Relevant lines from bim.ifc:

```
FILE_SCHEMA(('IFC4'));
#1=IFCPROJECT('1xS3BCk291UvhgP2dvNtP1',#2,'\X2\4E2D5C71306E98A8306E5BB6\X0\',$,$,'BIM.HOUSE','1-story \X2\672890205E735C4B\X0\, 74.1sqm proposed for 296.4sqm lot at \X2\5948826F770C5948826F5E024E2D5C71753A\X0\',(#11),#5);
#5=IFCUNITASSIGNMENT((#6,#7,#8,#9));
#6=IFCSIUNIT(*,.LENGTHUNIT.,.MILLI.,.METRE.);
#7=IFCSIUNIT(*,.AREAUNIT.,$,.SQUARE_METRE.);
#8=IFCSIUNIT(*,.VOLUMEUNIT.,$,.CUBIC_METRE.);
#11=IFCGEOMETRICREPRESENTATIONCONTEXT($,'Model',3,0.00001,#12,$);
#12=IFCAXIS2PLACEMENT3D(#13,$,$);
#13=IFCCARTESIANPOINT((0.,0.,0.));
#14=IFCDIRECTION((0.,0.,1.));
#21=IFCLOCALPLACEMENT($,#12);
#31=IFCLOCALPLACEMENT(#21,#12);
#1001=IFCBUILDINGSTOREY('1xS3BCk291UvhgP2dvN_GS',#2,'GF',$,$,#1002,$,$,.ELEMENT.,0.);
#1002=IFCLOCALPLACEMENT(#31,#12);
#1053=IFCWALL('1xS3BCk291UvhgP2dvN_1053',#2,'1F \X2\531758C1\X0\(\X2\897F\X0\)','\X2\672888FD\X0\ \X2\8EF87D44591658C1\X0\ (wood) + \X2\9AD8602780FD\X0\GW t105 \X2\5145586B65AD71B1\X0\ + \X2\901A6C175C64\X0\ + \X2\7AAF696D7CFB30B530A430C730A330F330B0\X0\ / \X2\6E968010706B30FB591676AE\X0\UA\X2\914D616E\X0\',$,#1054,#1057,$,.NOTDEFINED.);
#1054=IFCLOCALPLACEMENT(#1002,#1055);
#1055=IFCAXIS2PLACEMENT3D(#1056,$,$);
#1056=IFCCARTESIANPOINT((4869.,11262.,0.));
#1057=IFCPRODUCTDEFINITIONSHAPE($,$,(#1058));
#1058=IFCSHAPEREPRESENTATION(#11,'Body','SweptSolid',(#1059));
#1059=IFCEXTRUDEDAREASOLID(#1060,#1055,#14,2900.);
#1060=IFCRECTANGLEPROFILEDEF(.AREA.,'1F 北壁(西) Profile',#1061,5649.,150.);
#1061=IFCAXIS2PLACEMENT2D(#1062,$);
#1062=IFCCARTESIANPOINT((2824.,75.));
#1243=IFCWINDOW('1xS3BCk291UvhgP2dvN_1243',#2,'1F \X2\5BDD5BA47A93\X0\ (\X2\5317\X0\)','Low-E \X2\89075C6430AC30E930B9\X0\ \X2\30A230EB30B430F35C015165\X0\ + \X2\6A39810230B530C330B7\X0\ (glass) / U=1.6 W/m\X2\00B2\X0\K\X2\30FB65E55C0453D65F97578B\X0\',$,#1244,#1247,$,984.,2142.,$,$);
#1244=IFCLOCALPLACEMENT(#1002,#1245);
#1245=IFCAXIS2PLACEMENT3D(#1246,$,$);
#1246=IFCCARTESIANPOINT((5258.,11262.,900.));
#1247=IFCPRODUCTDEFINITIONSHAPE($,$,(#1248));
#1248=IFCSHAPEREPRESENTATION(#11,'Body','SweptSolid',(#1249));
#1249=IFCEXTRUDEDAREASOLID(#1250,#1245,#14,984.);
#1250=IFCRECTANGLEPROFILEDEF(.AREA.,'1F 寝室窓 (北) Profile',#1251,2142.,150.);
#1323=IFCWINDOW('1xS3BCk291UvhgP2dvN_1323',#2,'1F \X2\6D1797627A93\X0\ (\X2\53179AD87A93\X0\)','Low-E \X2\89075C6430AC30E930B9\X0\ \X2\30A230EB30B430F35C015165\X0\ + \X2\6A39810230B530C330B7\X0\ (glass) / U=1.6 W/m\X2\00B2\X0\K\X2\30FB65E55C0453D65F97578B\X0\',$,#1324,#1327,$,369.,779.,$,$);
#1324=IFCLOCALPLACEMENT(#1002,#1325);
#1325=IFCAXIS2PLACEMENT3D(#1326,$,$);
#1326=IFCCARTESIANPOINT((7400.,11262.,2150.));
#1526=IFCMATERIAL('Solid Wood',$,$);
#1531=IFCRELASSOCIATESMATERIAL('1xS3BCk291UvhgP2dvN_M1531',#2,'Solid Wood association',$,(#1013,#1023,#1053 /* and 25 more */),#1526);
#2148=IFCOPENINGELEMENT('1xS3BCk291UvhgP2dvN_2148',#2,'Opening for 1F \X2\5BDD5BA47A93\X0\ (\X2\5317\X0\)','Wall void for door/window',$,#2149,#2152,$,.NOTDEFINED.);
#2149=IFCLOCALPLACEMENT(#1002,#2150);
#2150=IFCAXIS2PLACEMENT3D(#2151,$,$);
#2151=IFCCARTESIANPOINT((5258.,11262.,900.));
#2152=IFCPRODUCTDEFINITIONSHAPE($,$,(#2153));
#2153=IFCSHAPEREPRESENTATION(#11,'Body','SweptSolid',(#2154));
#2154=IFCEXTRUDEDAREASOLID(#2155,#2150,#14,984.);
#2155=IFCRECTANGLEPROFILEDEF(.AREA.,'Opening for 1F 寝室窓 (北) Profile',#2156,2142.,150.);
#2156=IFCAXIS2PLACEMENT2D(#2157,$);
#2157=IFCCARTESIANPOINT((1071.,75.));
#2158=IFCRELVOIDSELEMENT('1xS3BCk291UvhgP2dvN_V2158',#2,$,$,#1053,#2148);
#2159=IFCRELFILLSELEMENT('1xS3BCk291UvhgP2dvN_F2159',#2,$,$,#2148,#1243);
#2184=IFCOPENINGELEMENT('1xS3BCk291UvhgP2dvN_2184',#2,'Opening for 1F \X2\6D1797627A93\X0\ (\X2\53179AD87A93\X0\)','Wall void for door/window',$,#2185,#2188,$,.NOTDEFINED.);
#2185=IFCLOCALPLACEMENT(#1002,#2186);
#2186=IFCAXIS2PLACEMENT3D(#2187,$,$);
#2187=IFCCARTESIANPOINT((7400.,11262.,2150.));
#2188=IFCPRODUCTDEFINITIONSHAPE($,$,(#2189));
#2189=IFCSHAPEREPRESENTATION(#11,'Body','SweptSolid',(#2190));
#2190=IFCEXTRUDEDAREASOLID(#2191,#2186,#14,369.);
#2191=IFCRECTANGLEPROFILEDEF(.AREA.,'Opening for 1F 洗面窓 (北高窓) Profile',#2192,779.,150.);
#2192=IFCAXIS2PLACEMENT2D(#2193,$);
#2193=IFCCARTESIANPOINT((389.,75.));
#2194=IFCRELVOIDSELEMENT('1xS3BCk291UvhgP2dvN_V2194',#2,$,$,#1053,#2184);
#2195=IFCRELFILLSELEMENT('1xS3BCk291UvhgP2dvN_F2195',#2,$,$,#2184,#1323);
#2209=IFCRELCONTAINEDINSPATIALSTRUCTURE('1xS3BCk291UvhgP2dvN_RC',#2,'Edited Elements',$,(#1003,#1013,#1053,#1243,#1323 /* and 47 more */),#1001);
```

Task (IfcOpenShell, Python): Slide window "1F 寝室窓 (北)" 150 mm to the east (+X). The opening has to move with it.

```python
import ifcopenshell
import ifcopenshell.api.geometry
import ifcopenshell.util.placement
import ifcopenshell.util.unit

model = ifcopenshell.open("bim.ifc")
unit_scale = ifcopenshell.util.unit.calculate_unit_scale(model)

window = model.by_guid("1xS3BCk291UvhgP2dvN_1243")
opening = window.FillsVoids[0].RelatingOpeningElement
wall = opening.VoidsElements[0].RelatingBuildingElement

wall_matrix = ifcopenshell.util.placement.get_local_placement(wall.ObjectPlacement)
shift = wall_matrix[:3, 0] * 0.15 / unit_scale
before = ifcopenshell.util.placement.get_local_placement(window.ObjectPlacement)[:3, 3].copy()

# The window is not placed relative to its opening, so move both.
for product in (opening, window):
    matrix = ifcopenshell.util.placement.get_local_placement(product.ObjectPlacement)
    matrix[:3, 3] += shift
    ifcopenshell.api.geometry.edit_object_placement(model, product=product, matrix=matrix, is_si=False)

after = ifcopenshell.util.placement.get_local_placement(window.ObjectPlacement)[:3, 3]
print("window moved by", (after - before).round(3) + 0.0)

model.write("bim_updated.ifc")
```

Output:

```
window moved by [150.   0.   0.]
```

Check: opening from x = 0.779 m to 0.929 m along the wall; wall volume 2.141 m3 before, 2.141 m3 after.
